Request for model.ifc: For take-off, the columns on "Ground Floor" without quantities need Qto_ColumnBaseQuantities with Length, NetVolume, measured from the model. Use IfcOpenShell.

First a look at what the model holds.

```python
import ifcopenshell
import ifcopenshell.util.element
import ifcopenshell.util.unit

model = ifcopenshell.open("model.ifc")
print(model.schema)
for unit_type in ("LENGTHUNIT", "AREAUNIT", "VOLUMEUNIT"):
    print(unit_type, ifcopenshell.util.unit.calculate_unit_scale(model, unit_type))
storey = next(s for s in model.by_type("IfcBuildingStorey") if s.Name == "Ground Floor")
columns = [e for e in ifcopenshell.util.element.get_decomposition(storey) if e.is_a("IfcColumn")]
for e in sorted(columns, key=lambda e: e.id()):
    print(e.id(), e.is_a(), e.Name, list(ifcopenshell.util.element.get_psets(e, qtos_only=True)), sep=" | ")
```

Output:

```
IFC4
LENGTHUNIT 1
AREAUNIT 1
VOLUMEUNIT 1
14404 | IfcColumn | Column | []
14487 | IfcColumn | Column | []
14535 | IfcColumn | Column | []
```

```python
import ifcopenshell
import ifcopenshell.api.pset
import ifcopenshell.geom
import ifcopenshell.util.element
import ifcopenshell.util.shape
import ifcopenshell.util.unit

model = ifcopenshell.open("model.ifc")
unit_scale = ifcopenshell.util.unit.calculate_unit_scale(model)
volume_scale = ifcopenshell.util.unit.calculate_unit_scale(model, "VOLUMEUNIT")
settings = ifcopenshell.geom.settings()

storey = next(s for s in model.by_type("IfcBuildingStorey") if s.Name == "Ground Floor")
columns = [e for e in ifcopenshell.util.element.get_decomposition(storey) if e.is_a("IfcColumn")]

for e in sorted(columns, key=lambda e: e.id()):
    if ifcopenshell.util.element.get_psets(e, qtos_only=True, should_inherit=False):
        continue
    # Geometry comes back in metres, in the element's own axes.
    shape = ifcopenshell.geom.create_shape(settings, e)
    values = {
        "Length": ifcopenshell.util.shape.get_z(shape.geometry) / unit_scale,
        "NetVolume": ifcopenshell.util.shape.get_volume(shape.geometry) / volume_scale,
    }
    qto = ifcopenshell.api.pset.add_qto(model, product=e, name="Qto_ColumnBaseQuantities")
    ifcopenshell.api.pset.edit_qto(model, qto=qto, properties=values)
    print(e.id(), {k: round(v, 3) for k, v in values.items()})

model.write("model_v2.ifc")
```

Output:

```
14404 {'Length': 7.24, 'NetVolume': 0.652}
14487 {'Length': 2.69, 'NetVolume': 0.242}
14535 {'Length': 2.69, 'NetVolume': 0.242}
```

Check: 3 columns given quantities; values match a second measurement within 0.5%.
